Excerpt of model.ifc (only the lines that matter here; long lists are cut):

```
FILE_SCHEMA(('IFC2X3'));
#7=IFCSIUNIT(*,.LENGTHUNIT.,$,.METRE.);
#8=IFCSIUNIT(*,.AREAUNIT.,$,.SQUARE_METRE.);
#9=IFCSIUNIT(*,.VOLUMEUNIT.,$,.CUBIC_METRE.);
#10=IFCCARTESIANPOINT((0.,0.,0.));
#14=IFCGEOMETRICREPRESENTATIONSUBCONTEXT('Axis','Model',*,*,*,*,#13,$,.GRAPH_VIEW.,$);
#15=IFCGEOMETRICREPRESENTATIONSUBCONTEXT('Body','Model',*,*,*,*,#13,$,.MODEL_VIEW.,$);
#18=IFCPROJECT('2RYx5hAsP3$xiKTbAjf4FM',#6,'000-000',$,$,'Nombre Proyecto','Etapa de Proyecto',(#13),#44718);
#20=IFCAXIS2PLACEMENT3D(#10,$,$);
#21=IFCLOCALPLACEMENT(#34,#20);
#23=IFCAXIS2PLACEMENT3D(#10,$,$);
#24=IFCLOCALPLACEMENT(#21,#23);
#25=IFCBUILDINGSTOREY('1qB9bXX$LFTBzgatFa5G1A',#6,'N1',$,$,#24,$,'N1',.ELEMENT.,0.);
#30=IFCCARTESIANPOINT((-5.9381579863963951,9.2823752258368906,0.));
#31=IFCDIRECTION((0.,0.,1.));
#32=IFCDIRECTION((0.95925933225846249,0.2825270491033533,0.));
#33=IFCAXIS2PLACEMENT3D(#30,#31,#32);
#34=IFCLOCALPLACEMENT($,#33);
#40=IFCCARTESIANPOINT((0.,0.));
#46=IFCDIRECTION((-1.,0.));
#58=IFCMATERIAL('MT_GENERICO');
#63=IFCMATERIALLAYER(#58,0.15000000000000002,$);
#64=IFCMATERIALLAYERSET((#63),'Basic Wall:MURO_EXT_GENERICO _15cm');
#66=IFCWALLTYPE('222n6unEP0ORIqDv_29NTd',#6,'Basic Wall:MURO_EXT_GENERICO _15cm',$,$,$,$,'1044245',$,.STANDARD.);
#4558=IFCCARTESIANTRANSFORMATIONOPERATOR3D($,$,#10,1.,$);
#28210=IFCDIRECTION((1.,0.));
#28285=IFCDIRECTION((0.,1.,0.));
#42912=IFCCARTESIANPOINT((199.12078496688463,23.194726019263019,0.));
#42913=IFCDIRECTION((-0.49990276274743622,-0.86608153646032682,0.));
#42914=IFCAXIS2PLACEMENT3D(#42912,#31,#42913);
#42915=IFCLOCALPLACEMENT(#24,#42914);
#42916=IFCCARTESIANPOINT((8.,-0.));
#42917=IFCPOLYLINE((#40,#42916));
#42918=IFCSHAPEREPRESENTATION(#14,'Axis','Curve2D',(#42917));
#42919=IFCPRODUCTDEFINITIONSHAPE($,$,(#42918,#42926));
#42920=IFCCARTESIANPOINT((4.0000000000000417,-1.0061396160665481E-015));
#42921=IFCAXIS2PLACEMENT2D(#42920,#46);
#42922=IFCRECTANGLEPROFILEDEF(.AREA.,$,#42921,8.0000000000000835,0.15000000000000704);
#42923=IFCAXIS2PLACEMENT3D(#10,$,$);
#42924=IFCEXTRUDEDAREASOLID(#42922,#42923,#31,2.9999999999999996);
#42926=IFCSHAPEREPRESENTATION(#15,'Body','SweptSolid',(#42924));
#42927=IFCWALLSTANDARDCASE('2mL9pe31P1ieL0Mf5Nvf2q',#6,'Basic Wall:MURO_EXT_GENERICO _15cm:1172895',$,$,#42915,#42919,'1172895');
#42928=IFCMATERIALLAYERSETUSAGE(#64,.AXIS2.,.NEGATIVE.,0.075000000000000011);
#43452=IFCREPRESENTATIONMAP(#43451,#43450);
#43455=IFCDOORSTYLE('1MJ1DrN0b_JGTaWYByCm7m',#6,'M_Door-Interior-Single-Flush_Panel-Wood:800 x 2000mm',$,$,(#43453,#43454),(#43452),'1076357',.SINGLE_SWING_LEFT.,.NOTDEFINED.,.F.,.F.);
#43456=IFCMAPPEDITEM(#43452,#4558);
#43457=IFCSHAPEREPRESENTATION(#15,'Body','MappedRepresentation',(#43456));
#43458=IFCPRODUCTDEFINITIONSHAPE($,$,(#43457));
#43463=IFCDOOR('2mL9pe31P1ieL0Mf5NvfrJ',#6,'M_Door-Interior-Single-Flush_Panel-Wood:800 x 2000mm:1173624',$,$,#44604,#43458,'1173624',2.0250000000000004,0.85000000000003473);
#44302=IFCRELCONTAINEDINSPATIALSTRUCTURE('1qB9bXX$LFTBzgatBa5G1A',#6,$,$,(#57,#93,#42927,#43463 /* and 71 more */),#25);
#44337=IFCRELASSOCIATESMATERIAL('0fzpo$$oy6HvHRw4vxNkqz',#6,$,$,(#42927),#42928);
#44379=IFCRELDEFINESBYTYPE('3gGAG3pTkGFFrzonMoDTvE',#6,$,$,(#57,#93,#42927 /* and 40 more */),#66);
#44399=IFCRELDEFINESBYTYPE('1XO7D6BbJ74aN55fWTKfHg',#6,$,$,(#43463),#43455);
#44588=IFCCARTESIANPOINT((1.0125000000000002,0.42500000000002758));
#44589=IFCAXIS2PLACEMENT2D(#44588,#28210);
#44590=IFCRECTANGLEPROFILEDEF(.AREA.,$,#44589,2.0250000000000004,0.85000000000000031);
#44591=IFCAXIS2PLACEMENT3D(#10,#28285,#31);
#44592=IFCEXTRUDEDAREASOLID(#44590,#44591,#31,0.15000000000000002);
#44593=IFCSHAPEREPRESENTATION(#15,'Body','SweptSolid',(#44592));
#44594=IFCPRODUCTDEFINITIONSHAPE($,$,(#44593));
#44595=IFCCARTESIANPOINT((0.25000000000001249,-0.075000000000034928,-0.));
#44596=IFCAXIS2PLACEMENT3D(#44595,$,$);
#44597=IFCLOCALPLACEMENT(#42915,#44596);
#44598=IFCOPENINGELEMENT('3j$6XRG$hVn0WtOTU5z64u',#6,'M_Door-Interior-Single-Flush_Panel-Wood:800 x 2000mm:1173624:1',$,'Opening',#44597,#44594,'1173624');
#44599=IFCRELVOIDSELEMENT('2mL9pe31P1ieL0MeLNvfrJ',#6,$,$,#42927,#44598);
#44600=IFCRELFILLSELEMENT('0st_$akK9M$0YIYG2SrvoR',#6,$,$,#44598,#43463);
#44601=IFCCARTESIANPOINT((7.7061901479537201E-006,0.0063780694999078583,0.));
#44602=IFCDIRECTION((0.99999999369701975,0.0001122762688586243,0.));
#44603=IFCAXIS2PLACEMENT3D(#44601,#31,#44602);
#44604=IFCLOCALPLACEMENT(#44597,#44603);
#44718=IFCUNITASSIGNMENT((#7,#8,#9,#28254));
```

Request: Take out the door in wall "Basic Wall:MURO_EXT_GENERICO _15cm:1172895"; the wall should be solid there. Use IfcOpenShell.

```python
import ifcopenshell
import ifcopenshell.api.feature
import ifcopenshell.api.root
import ifcopenshell.geom
import ifcopenshell.util.shape

model = ifcopenshell.open("model.ifc")
settings = ifcopenshell.geom.settings()


def volume(element):
    """Net volume in cubic metres, openings subtracted."""
    shape = ifcopenshell.geom.create_shape(settings, element)
    return ifcopenshell.util.shape.get_volume(shape.geometry)


door = model.by_id(43463)
opening = door.FillsVoids[0].RelatingOpeningElement
wall = opening.VoidsElements[0].RelatingBuildingElement
before = volume(wall)

ifcopenshell.api.root.remove_product(model, product=door)
ifcopenshell.api.feature.remove_feature(model, feature=opening)

after = volume(wall)

print(f"wall volume {before:.3f} -> {after:.3f} m3")

model.write("model_updated.ifc")
```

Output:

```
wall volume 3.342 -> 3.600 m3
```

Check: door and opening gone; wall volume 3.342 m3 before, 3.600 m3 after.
